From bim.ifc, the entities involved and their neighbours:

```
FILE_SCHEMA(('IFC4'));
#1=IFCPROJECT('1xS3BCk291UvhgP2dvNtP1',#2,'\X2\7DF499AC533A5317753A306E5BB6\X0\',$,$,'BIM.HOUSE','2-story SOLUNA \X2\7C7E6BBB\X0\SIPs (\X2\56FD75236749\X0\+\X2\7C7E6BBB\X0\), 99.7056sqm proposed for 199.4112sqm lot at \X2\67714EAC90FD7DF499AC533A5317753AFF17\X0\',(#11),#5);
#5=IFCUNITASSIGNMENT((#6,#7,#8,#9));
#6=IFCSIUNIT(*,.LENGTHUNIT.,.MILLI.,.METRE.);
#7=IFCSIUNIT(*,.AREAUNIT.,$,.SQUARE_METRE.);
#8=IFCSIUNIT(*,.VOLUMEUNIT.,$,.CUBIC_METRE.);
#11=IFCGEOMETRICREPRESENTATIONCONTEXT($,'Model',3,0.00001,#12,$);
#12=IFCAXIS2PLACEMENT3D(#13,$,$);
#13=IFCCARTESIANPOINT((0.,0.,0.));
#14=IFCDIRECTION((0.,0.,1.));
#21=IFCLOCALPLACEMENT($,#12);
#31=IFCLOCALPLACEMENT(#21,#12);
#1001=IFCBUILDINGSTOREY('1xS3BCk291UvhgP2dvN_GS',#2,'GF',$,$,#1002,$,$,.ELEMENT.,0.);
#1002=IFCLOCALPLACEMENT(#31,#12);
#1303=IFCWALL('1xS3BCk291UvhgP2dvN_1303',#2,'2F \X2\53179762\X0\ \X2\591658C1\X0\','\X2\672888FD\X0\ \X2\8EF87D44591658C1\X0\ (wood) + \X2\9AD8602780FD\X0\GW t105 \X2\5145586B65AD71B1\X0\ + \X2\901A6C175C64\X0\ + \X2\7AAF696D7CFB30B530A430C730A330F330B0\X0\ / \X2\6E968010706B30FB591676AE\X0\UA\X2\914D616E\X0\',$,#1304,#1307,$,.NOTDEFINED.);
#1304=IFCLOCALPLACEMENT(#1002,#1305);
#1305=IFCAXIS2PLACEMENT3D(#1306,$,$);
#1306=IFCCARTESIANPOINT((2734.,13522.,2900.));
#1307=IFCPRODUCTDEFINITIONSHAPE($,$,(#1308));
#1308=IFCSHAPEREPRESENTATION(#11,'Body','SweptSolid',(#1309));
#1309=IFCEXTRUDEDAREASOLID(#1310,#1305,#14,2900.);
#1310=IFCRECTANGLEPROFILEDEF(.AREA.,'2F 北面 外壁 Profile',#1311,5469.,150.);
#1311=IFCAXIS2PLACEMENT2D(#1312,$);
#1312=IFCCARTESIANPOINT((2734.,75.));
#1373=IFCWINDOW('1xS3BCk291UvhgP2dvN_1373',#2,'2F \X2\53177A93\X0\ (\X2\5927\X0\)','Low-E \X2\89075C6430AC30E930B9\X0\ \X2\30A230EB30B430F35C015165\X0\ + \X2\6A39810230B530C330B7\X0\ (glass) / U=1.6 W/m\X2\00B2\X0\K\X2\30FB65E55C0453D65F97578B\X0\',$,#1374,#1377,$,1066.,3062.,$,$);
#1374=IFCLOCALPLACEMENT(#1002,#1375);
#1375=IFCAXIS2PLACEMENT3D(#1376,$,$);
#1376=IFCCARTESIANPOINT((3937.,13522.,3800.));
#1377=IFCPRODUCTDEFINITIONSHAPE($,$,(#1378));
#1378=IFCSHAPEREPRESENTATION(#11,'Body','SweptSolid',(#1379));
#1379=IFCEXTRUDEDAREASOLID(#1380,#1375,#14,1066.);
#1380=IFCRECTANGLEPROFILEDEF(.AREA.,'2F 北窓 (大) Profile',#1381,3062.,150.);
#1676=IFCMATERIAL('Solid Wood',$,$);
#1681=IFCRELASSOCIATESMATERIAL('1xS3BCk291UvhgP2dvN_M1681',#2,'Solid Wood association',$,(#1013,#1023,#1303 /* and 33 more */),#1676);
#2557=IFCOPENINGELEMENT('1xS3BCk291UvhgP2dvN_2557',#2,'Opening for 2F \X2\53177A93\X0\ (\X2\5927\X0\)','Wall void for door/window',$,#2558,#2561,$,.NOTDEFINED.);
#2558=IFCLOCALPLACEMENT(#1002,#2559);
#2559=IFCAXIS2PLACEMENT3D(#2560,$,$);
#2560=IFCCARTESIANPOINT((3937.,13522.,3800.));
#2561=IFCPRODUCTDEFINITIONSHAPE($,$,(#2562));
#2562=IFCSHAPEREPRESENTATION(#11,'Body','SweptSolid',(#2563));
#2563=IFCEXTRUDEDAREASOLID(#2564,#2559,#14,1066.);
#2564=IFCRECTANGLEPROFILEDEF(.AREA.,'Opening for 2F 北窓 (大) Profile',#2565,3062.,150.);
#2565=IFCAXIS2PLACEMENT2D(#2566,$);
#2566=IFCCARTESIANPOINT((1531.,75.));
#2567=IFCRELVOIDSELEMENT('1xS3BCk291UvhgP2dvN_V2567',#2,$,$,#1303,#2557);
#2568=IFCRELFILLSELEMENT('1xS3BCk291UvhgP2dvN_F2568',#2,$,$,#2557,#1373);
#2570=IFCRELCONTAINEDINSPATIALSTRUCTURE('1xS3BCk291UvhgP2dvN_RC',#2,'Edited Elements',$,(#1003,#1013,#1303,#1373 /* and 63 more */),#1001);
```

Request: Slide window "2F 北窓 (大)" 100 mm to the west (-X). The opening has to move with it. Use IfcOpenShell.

```python
import ifcopenshell
import ifcopenshell.api.geometry
import ifcopenshell.util.placement
import ifcopenshell.util.unit

model = ifcopenshell.open("bim.ifc")
unit_scale = ifcopenshell.util.unit.calculate_unit_scale(model)

window = model.by_id(1373)
opening = window.FillsVoids[0].RelatingOpeningElement
wall = opening.VoidsElements[0].RelatingBuildingElement

wall_matrix = ifcopenshell.util.placement.get_local_placement(wall.ObjectPlacement)
shift = wall_matrix[:3, 0] * -0.1 / unit_scale
before = ifcopenshell.util.placement.get_local_placement(window.ObjectPlacement)[:3, 3].copy()

# The window is not placed relative to its opening, so move both.
for product in (opening, window):
    matrix = ifcopenshell.util.placement.get_local_placement(product.ObjectPlacement)
    matrix[:3, 3] += shift
    ifcopenshell.api.geometry.edit_object_placement(model, product=product, matrix=matrix, is_si=False)

after = ifcopenshell.util.placement.get_local_placement(window.ObjectPlacement)[:3, 3]
print("window moved by", (after - before).round(3) + 0.0)

model.write("bim_edited.ifc")
```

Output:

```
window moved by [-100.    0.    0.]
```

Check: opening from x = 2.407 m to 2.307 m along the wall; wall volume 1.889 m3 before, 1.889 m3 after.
